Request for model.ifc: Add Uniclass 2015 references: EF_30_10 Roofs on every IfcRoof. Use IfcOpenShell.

First a look at what the model holds.

```python
import ifcopenshell

model = ifcopenshell.open("model.ifc")
print(model.schema)
print("classifications:", [c.Name for c in model.by_type("IfcClassification")])
for ifc_class in ("IfcDoor", "IfcRoof", "IfcStair", "IfcWall", "IfcWindow"):
    print(ifc_class, len(model.by_type(ifc_class)))
```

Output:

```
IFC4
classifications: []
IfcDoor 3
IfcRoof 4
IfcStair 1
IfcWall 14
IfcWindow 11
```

```python
import ifcopenshell
import ifcopenshell.api.classification

model = ifcopenshell.open("model.ifc")

system = ifcopenshell.api.classification.add_classification(model, classification="Uniclass 2015")

codes = {
    "IfcRoof": ("EF_30_10", "Roofs"),
}
for ifc_class, (code, name) in codes.items():
    products = model.by_type(ifc_class)
    ifcopenshell.api.classification.add_reference(
        model, products=products, classification=system, identification=code, name=name
    )
    print(code, len(products))

model.write("model-out.ifc")
```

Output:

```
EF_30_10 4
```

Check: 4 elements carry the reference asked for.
